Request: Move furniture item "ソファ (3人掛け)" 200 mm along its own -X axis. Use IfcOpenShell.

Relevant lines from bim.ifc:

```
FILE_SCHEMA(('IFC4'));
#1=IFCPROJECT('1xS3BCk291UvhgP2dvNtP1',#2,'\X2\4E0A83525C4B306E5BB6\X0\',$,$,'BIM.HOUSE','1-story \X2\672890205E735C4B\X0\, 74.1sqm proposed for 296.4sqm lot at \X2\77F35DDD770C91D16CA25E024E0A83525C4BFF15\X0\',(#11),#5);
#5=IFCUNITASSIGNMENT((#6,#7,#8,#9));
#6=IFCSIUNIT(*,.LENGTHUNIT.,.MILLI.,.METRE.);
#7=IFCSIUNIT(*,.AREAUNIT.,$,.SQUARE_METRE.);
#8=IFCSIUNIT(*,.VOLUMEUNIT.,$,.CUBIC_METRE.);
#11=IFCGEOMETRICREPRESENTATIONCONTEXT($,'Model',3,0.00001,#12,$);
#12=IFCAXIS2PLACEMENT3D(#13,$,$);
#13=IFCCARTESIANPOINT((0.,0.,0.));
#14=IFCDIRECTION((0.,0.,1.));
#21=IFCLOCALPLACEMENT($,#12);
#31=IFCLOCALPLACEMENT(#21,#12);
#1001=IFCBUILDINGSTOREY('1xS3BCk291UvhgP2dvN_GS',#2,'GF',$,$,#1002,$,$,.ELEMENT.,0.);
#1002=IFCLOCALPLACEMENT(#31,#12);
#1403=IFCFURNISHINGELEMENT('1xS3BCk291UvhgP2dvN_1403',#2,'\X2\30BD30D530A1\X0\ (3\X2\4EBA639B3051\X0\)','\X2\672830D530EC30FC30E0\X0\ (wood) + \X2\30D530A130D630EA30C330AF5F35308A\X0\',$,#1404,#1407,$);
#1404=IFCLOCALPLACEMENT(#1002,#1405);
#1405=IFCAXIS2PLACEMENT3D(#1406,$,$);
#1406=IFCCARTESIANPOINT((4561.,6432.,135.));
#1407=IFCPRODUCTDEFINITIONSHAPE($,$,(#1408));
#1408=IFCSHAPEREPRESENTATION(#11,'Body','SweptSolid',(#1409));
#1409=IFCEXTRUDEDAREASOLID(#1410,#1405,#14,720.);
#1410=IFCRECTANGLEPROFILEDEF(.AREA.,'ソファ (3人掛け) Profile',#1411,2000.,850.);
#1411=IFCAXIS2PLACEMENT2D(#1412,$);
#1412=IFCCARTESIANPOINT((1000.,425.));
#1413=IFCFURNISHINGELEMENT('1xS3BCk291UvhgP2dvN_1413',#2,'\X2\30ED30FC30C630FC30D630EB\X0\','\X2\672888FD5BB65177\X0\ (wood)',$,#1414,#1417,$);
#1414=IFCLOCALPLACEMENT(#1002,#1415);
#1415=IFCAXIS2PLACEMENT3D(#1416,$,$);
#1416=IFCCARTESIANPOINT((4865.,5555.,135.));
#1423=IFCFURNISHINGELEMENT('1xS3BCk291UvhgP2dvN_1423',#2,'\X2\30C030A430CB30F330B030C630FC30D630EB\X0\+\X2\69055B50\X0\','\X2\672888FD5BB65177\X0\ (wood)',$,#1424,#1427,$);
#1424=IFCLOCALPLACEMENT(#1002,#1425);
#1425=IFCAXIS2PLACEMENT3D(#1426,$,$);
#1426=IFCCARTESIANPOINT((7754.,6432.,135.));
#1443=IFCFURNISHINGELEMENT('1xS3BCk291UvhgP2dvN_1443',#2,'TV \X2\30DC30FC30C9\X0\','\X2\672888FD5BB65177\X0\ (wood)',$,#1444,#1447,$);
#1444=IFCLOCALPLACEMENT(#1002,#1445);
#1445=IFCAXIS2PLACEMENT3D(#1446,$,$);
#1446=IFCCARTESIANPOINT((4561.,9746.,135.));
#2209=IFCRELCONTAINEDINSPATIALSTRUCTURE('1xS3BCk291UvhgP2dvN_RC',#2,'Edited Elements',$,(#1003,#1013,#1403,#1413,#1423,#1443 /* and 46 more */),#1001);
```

```python
import ifcopenshell
import ifcopenshell.api.geometry
import ifcopenshell.util.placement

model = ifcopenshell.open("bim.ifc")

item = model.by_id(1403)
matrix = ifcopenshell.util.placement.get_local_placement(item.ObjectPlacement)
matrix[:3, 3] -= matrix[:3, 0] * 200.0
ifcopenshell.api.geometry.edit_object_placement(model, product=item, matrix=matrix, is_si=False)

print(ifcopenshell.util.placement.get_local_placement(item.ObjectPlacement).round(3) + 0.0)

model.write("bim_edited.ifc")
```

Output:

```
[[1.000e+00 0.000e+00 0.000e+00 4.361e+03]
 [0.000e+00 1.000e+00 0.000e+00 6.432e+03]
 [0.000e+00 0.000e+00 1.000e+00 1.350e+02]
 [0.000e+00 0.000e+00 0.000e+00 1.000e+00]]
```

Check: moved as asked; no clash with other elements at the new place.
